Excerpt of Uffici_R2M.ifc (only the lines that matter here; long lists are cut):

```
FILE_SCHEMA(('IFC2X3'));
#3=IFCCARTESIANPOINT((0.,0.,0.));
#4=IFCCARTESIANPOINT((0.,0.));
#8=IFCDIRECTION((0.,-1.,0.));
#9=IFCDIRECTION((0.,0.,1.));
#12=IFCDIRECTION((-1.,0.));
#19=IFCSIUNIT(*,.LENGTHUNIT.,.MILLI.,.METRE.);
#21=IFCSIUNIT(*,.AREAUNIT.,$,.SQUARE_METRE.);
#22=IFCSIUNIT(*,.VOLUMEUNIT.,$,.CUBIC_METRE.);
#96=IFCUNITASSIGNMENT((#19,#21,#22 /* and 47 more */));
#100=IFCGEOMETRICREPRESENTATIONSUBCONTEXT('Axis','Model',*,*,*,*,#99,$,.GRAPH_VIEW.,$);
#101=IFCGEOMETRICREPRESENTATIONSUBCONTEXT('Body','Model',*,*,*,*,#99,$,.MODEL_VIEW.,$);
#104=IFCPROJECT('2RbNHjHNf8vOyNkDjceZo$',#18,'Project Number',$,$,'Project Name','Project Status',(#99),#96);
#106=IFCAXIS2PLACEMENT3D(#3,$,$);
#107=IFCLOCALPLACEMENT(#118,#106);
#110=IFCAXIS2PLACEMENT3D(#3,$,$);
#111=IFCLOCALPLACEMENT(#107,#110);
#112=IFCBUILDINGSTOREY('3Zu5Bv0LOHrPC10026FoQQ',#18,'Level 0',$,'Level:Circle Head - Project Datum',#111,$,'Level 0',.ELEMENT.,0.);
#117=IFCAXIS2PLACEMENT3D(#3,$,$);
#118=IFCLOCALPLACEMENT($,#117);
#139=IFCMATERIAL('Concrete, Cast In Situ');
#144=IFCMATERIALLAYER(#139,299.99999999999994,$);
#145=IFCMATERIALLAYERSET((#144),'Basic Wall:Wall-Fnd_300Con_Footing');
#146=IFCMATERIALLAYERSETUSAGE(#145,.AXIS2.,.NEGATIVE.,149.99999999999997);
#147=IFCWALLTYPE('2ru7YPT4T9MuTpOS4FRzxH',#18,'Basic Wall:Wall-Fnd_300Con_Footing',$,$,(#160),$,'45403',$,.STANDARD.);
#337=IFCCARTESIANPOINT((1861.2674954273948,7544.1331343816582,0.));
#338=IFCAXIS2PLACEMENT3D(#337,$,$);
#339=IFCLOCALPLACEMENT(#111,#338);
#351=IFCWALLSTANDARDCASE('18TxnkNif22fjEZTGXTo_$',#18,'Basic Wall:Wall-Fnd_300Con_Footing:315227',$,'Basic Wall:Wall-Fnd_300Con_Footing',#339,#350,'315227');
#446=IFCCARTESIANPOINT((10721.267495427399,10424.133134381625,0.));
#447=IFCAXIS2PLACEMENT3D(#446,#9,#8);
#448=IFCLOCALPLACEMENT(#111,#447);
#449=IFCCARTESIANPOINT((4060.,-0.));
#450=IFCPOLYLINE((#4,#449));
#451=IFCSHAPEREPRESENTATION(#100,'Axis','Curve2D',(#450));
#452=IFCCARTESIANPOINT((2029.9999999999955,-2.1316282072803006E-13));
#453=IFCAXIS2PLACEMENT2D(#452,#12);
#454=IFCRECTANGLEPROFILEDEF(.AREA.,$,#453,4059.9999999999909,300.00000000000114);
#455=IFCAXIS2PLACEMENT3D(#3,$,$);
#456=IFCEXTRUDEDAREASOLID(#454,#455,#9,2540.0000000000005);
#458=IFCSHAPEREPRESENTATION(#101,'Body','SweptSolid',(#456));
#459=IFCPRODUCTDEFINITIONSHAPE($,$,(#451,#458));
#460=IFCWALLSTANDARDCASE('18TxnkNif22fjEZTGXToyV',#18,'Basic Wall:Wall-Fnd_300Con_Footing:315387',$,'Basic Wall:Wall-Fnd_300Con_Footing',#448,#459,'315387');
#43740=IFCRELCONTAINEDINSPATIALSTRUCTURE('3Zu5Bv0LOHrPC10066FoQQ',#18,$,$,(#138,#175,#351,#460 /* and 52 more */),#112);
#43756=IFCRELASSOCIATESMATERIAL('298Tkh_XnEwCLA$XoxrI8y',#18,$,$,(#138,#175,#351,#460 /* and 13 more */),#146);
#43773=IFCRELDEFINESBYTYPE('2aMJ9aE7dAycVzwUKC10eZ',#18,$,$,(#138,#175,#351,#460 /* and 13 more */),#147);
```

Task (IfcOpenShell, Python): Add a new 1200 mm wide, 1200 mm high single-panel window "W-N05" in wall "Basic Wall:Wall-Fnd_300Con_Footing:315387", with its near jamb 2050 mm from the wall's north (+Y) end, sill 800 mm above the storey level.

```python
import numpy as np
import ifcopenshell
import ifcopenshell.api.feature
import ifcopenshell.api.geometry
import ifcopenshell.api.root
import ifcopenshell.api.spatial
import ifcopenshell.api.type
import ifcopenshell.geom
import ifcopenshell.util.element
import ifcopenshell.util.placement
import ifcopenshell.util.representation
import ifcopenshell.util.shape
import ifcopenshell.util.unit

model = ifcopenshell.open("Uffici_R2M.ifc")
unit_scale = ifcopenshell.util.unit.calculate_unit_scale(model)
settings = ifcopenshell.geom.settings()


def volume(element):
    """Net volume in cubic metres, openings subtracted."""
    shape = ifcopenshell.geom.create_shape(settings, element)
    return ifcopenshell.util.shape.get_volume(shape.geometry)


wall = model.by_guid("18TxnkNif22fjEZTGXToyV")
storey = ifcopenshell.util.element.get_container(wall, ifc_class="IfcBuildingStorey")
context = ifcopenshell.util.representation.get_context(model, "Model", "Body", "MODEL_VIEW")
before = volume(wall)

width, height, from_end, sill = 1.2, 1.2, 2.05, 0.8  # metres

# The wall runs along its own X axis, and the end named is its -X end.
wall_shape = ifcopenshell.geom.create_shape(settings, wall)
x, y, z = ifcopenshell.util.shape.get_vertices(wall_shape.geometry).T
start = x.min() + from_end
face, thickness = float(y.min()), float(y.max() - y.min())
wall_matrix = ifcopenshell.util.placement.get_local_placement(wall.ObjectPlacement)
level = ifcopenshell.util.placement.get_local_placement(storey.ObjectPlacement)[2, 3]


def in_wall(x, y):
    """Placement at x, y metres in the wall's axes, at sill height."""
    matrix = wall_matrix.copy()
    matrix[:, 3] = wall_matrix @ np.array([x / unit_scale, y / unit_scale, 0.0, 1.0])
    matrix[2, 3] = level + sill / unit_scale
    return matrix


# Opening: a box that overshoots both wall faces by 50 mm.
opening = ifcopenshell.api.root.create_entity(model, ifc_class="IfcOpeningElement")
box = ifcopenshell.api.geometry.add_wall_representation(
    model, context=context, length=width, height=height, thickness=thickness + 0.1
)
ifcopenshell.api.geometry.assign_representation(model, product=opening, representation=box)
ifcopenshell.api.geometry.edit_object_placement(model, product=opening, matrix=in_wall(start, face - 0.05), is_si=False)
ifcopenshell.api.feature.add_feature(model, feature=opening, element=wall)

window = ifcopenshell.api.root.create_entity(model, ifc_class="IfcWindow", name="W-N05")
window.OverallWidth, window.OverallHeight = width / unit_scale, height / unit_scale
body = ifcopenshell.api.geometry.add_window_representation(
    model,
    context=context,
    overall_width=window.OverallWidth,
    overall_height=window.OverallHeight,
    partition_type="SINGLE_PANEL",
)
ifcopenshell.api.geometry.assign_representation(model, product=window, representation=body)
ifcopenshell.api.spatial.assign_container(model, products=[window], relating_structure=storey)
fills = ifcopenshell.api.feature.add_filling(model, opening=opening, element=window)
fills.OwnerHistory = window.OwnerHistory  # required in IFC2X3

# IFC2X3 keeps the operation on the window style.
style = ifcopenshell.api.root.create_entity(model, ifc_class="IfcWindowStyle", name="W-N05")
style.OperationType, style.ConstructionType = "SINGLE_PANEL", "NOTDEFINED"
style.ParameterTakesPrecedence = style.Sizeable = False
ifcopenshell.api.type.assign_type(model, related_objects=[window], relating_type=style)

# Centre the window in the wall's thickness.
ifcopenshell.api.geometry.edit_object_placement(model, product=window, matrix=in_wall(start, face), is_si=False)
window_shape = ifcopenshell.geom.create_shape(settings, window)
depth = ifcopenshell.util.shape.get_vertices(window_shape.geometry)[:, 1]
offset = face + thickness / 2 - (depth.min() + depth.max()) / 2
ifcopenshell.api.geometry.edit_object_placement(model, product=window, matrix=in_wall(start, offset), is_si=False)

after = volume(wall)

print(f"wall volume {before:.3f} -> {after:.3f} m3")

model.write("Uffici_R2M_v2.ifc")
```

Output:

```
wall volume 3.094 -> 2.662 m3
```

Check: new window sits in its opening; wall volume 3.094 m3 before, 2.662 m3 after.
